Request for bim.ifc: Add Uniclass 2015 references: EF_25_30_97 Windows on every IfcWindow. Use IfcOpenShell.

First a look at what the model holds.

```python
import ifcopenshell

model = ifcopenshell.open("bim.ifc")
print(model.schema)
print("classifications:", [c.Name for c in model.by_type("IfcClassification")])
for ifc_class in ("IfcDoor", "IfcRoof", "IfcStair", "IfcWall", "IfcWindow"):
    print(ifc_class, len(model.by_type(ifc_class)))
```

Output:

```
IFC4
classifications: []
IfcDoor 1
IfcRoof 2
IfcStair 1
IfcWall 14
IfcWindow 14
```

```python
import ifcopenshell
import ifcopenshell.api.classification

model = ifcopenshell.open("bim.ifc")

system = ifcopenshell.api.classification.add_classification(model, classification="Uniclass 2015")

codes = {
    "IfcWindow": ("EF_25_30_97", "Windows"),
}
for ifc_class, (code, name) in codes.items():
    products = model.by_type(ifc_class)
    ifcopenshell.api.classification.add_reference(
        model, products=products, classification=system, identification=code, name=name
    )
    print(code, len(products))

model.write("bim_rev.ifc")
```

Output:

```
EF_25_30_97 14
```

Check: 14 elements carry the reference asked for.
